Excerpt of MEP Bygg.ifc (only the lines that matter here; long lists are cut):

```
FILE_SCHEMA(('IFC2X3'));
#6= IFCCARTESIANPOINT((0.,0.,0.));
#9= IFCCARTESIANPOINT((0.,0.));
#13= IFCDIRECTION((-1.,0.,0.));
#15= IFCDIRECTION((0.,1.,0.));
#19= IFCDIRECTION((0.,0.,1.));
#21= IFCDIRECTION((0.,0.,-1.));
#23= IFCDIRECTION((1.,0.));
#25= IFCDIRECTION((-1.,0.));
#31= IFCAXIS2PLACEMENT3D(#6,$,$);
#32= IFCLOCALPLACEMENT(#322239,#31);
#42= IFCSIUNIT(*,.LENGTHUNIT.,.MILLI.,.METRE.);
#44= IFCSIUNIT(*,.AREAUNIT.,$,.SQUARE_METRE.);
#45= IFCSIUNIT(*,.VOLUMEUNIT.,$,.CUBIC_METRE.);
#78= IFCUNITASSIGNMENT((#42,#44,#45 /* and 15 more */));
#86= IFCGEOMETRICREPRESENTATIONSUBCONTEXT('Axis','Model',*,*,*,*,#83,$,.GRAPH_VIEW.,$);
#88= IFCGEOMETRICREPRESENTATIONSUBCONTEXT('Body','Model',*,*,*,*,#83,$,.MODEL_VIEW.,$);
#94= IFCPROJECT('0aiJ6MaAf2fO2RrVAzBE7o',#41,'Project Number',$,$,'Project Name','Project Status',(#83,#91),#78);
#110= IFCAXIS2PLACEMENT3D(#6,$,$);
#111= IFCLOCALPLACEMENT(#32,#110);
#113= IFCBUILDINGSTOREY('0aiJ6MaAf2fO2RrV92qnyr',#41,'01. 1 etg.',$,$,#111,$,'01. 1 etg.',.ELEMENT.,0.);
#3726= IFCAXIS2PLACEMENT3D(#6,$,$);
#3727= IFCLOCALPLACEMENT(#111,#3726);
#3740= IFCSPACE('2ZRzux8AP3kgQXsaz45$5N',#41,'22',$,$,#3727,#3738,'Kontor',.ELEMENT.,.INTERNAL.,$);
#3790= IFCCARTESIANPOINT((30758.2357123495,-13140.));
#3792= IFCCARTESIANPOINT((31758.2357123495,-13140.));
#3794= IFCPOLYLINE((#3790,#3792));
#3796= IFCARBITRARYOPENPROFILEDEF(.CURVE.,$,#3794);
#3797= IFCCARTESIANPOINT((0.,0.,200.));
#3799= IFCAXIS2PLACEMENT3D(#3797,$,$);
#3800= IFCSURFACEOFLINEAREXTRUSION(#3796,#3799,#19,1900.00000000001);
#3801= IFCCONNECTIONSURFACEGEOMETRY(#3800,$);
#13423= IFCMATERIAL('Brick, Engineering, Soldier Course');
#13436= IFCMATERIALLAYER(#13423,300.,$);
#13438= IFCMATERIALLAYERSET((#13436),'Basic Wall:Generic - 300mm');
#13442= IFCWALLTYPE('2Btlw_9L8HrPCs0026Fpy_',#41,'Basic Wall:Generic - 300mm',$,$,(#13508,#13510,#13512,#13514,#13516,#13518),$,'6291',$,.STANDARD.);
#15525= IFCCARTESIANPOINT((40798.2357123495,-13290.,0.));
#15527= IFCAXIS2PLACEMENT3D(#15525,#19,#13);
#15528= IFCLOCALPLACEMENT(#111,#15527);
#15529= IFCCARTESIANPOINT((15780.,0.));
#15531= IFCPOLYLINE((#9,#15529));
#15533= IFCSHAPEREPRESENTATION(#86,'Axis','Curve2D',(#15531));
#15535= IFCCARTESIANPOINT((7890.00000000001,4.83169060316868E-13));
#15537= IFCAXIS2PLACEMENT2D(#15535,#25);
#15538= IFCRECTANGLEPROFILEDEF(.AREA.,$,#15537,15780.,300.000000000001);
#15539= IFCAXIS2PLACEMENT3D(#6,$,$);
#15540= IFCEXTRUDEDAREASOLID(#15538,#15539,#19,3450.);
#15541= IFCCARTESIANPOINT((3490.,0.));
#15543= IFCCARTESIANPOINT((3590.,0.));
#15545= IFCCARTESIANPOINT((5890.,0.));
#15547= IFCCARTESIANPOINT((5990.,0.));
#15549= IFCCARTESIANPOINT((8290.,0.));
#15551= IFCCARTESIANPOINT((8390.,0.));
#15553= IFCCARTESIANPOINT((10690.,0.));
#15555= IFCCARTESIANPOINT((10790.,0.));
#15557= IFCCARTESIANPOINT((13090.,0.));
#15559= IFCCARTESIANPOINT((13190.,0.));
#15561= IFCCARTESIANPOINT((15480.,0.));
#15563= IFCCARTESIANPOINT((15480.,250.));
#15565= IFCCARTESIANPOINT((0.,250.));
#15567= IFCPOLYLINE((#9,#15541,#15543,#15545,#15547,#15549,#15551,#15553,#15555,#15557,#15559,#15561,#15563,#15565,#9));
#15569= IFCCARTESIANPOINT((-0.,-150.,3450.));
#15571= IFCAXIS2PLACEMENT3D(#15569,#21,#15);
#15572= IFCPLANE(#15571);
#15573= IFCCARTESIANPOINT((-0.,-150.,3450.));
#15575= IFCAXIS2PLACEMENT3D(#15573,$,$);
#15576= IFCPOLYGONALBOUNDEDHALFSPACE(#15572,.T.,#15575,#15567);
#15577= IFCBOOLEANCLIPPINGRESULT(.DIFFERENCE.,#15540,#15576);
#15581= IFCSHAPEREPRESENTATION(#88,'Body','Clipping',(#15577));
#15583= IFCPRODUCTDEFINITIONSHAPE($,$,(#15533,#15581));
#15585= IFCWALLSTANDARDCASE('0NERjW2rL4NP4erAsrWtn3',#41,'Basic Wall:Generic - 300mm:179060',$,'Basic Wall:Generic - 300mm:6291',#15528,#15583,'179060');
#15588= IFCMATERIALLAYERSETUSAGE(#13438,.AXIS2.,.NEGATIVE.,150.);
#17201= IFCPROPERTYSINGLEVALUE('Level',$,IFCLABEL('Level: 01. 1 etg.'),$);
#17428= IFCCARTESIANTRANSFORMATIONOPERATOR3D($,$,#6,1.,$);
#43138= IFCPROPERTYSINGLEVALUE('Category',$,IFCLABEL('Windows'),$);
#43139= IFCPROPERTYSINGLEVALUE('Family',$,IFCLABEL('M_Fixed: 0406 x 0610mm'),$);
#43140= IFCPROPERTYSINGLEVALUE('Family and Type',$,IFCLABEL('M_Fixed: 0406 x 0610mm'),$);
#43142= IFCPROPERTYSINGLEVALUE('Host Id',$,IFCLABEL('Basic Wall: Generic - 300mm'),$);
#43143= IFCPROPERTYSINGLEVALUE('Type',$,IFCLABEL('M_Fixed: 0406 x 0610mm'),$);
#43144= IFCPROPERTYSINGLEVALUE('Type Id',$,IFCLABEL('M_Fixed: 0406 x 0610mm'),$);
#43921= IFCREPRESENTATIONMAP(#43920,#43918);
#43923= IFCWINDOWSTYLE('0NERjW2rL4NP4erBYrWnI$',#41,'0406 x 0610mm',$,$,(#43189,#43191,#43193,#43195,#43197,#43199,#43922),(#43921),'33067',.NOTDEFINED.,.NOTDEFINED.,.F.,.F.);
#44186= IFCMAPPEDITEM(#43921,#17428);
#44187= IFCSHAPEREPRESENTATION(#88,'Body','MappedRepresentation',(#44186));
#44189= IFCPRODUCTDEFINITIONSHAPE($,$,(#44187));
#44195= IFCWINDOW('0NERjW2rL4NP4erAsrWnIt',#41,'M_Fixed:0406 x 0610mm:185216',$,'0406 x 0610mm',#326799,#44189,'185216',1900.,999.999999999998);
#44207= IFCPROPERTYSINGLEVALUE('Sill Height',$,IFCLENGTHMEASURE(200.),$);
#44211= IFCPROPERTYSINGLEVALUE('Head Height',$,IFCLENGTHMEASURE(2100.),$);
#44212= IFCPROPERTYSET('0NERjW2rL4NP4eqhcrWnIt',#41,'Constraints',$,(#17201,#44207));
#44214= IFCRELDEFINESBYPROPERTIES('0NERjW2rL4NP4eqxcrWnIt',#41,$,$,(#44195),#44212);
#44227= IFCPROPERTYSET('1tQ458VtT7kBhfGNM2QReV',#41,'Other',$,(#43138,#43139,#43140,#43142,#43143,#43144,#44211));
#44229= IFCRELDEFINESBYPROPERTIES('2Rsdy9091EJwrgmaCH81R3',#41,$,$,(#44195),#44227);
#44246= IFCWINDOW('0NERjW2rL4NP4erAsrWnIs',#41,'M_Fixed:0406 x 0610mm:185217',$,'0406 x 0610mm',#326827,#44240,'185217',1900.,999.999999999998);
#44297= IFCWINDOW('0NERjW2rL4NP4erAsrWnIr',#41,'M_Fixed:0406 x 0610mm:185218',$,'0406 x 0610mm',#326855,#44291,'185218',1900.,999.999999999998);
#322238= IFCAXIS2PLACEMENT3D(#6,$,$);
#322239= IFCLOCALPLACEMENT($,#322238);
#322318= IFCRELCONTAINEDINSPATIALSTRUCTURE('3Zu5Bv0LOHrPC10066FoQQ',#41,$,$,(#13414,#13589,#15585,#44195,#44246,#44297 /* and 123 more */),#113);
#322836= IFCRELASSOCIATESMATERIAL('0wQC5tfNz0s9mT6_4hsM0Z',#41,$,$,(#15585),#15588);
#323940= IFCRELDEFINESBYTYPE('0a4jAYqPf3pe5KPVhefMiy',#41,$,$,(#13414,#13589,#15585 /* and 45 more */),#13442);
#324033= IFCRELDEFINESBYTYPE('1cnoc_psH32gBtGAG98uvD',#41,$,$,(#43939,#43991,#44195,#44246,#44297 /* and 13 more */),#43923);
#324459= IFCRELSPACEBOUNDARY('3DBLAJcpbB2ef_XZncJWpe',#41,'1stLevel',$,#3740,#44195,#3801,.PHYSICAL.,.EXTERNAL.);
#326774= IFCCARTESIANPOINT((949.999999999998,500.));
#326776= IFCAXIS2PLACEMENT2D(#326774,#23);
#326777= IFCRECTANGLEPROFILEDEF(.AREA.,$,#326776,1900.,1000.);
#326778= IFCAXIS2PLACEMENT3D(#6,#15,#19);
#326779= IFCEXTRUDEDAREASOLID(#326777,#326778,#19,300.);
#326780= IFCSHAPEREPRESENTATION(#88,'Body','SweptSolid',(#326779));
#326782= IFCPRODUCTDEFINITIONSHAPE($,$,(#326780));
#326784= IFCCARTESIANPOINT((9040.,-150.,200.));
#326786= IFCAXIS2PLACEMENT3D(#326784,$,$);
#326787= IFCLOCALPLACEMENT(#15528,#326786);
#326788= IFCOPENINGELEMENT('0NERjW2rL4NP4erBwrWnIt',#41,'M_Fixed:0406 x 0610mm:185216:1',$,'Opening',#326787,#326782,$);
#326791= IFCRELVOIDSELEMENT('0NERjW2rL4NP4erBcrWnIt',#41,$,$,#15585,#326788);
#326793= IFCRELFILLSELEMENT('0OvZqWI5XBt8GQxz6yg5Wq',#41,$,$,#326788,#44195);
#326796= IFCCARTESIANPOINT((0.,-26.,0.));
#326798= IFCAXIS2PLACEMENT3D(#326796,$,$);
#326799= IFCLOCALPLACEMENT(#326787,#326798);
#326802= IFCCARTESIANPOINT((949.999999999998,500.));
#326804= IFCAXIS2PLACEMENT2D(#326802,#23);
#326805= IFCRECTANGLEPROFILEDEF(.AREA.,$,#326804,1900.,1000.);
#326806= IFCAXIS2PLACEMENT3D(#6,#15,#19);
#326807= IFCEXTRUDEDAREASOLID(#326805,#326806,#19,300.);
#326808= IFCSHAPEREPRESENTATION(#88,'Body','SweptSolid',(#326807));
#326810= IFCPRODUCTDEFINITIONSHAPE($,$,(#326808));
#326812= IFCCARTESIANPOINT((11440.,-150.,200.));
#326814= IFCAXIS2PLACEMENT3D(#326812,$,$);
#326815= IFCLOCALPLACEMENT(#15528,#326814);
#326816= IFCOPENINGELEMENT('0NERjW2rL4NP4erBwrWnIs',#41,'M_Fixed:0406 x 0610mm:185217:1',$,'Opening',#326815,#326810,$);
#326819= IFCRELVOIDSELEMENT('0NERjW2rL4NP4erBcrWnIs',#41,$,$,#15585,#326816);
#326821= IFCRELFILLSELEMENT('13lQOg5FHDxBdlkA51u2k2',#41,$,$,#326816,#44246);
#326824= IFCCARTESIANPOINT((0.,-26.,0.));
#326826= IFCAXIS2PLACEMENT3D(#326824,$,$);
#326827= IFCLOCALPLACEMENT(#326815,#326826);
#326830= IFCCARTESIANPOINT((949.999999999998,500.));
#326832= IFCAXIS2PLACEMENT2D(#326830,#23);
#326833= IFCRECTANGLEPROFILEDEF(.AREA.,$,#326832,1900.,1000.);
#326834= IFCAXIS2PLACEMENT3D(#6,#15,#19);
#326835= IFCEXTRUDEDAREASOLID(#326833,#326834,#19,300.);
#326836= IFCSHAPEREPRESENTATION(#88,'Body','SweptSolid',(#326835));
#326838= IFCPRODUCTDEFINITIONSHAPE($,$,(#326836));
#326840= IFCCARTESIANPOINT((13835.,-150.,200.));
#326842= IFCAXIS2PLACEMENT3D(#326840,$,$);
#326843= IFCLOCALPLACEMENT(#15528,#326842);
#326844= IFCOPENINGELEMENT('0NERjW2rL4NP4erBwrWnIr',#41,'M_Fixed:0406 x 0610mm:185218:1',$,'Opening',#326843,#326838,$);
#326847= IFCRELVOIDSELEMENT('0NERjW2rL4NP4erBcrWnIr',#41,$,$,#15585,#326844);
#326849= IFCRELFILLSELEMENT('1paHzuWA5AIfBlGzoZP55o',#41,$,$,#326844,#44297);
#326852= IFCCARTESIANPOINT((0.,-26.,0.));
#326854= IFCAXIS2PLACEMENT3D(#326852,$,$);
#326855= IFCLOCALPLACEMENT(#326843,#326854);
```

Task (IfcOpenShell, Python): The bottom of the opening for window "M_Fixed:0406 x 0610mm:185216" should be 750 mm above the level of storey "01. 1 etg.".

```python
import numpy as np
import ifcopenshell
import ifcopenshell.api.geometry
import ifcopenshell.api.pset
import ifcopenshell.geom
import ifcopenshell.util.element
import ifcopenshell.util.placement
import ifcopenshell.util.shape
import ifcopenshell.util.unit

model = ifcopenshell.open("MEP Bygg.ifc")
unit_scale = ifcopenshell.util.unit.calculate_unit_scale(model)

window = model.by_guid("0NERjW2rL4NP4erAsrWnIt")
opening = window.FillsVoids[0].RelatingOpeningElement
storey = ifcopenshell.util.element.get_container(window, ifc_class="IfcBuildingStorey")
level = ifcopenshell.util.placement.get_local_placement(storey.ObjectPlacement)[2, 3]

# The opening's origin need not be at the sill, so measure its lowest point.
shape = ifcopenshell.geom.create_shape(ifcopenshell.geom.settings(), opening)
bottom = ifcopenshell.util.shape.get_shape_bottom_elevation(shape, shape.geometry) / unit_scale
dz = level + 0.75 / unit_scale - bottom

shift = np.array([0.0, 0.0, dz])
# The window is placed relative to its opening, so it follows when the opening moves.
matrix = ifcopenshell.util.placement.get_local_placement(opening.ObjectPlacement)
matrix[:3, 3] += shift
ifcopenshell.api.geometry.edit_object_placement(
    model, product=opening, matrix=matrix, is_si=False, should_transform_children=True
)

# Space boundary surfaces are stored in each space's coordinates; move them too.
for rel in window.ProvidesBoundaries:
    if not rel.ConnectionGeometry:
        continue
    surface = rel.ConnectionGeometry.SurfaceOnRelatingElement
    space_matrix = ifcopenshell.util.placement.get_local_placement(rel.RelatingSpace.ObjectPlacement)
    point = np.array(surface.Position.Location.Coordinates) + space_matrix[:3, :3].T @ shift
    surface.Position = model.createIfcAxis2Placement3D(
        model.createIfcCartesianPoint(point.tolist()), surface.Position.Axis, surface.Position.RefDirection
    )

# Keep the stored heights in step.
pset = model.by_id(ifcopenshell.util.element.get_pset(window, "Constraints", should_inherit=False)["id"])
ifcopenshell.api.pset.edit_pset(model, pset=pset, properties={
    "Sill Height": model.create_entity("IfcLengthMeasure", ifcopenshell.util.element.get_pset(window, "Constraints", "Sill Height") + dz),
})
pset = model.by_id(ifcopenshell.util.element.get_pset(window, "Other", should_inherit=False)["id"])
ifcopenshell.api.pset.edit_pset(model, pset=pset, properties={
    "Head Height": model.create_entity("IfcLengthMeasure", ifcopenshell.util.element.get_pset(window, "Other", "Head Height") + dz),
})

print(f"moved by {dz * unit_scale:+.3f} m")

model.write("MEP Bygg_updated.ifc")
```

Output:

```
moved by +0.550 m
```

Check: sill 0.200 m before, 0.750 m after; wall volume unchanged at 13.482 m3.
